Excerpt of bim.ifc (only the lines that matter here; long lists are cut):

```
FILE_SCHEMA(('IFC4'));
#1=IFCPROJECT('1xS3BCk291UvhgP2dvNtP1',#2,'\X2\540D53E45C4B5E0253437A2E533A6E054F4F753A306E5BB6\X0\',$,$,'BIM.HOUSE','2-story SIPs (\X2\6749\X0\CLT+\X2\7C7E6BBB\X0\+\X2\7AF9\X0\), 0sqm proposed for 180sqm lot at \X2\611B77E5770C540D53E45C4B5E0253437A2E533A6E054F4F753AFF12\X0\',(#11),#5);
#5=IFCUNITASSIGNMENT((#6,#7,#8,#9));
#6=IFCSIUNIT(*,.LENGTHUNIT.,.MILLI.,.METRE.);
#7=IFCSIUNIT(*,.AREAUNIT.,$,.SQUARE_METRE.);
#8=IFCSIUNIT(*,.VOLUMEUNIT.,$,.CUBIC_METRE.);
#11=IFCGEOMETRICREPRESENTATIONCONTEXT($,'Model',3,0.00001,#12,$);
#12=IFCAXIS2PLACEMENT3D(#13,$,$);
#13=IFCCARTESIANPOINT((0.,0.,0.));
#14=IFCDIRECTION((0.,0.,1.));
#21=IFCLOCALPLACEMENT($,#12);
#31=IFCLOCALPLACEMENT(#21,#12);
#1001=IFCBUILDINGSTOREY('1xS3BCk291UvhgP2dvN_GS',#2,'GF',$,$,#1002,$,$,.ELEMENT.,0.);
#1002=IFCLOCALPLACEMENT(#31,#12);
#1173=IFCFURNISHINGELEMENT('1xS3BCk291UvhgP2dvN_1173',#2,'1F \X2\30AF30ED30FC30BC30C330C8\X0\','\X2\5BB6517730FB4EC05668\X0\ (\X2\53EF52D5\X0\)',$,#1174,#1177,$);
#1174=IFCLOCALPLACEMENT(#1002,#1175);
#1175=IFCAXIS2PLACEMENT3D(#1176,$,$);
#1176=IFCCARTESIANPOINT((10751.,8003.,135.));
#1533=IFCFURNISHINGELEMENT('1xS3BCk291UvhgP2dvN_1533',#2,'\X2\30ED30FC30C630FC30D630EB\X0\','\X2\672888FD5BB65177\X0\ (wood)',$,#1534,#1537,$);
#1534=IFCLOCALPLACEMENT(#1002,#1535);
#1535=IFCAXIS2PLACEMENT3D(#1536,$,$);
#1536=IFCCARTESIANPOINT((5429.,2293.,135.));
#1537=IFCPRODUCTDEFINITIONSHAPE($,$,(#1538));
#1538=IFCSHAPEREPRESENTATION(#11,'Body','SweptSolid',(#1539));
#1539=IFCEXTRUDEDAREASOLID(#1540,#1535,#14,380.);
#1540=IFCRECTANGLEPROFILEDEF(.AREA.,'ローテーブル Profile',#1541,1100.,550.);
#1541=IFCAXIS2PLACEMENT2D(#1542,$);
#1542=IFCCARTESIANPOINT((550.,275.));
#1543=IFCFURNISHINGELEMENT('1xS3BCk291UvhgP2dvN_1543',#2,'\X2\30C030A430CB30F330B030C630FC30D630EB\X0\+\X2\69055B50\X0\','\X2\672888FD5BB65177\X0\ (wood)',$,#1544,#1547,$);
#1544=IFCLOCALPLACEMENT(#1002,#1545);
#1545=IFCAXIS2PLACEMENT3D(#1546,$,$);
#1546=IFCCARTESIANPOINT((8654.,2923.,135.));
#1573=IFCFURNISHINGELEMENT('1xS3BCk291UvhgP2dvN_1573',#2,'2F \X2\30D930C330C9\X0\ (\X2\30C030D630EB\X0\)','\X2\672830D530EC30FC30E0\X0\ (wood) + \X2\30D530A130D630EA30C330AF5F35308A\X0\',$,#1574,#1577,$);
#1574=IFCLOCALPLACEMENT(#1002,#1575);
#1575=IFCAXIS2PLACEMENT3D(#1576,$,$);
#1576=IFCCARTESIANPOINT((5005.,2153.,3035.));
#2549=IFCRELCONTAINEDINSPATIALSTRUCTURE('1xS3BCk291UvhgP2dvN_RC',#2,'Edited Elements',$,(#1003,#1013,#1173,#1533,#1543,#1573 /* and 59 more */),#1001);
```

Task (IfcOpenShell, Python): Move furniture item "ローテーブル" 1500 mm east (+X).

```python
import ifcopenshell
import ifcopenshell.api.geometry
import ifcopenshell.util.placement
import ifcopenshell.util.unit

model = ifcopenshell.open("bim.ifc")
unit_scale = ifcopenshell.util.unit.calculate_unit_scale(model)

item = model.by_guid("1xS3BCk291UvhgP2dvN_1533")
matrix = ifcopenshell.util.placement.get_local_placement(item.ObjectPlacement)
matrix[0, 3] += 1.5 / unit_scale
ifcopenshell.api.geometry.edit_object_placement(model, product=item, matrix=matrix, is_si=False)

print(ifcopenshell.util.placement.get_local_placement(item.ObjectPlacement).round(3) + 0.0)

model.write("bim_v2.ifc")
```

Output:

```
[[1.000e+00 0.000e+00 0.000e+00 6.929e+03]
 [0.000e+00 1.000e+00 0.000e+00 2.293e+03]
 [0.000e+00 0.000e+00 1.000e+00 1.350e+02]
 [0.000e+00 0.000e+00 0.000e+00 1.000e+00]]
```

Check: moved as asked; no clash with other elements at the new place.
